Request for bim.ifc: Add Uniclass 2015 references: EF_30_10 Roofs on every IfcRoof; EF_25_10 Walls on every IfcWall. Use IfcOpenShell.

First a look at what the model holds.

```python
import ifcopenshell

model = ifcopenshell.open("bim.ifc")
print(model.schema)
print("classifications:", [c.Name for c in model.by_type("IfcClassification")])
for ifc_class in ("IfcDoor", "IfcRoof", "IfcStair", "IfcWall", "IfcWindow"):
    print(ifc_class, len(model.by_type(ifc_class)))
```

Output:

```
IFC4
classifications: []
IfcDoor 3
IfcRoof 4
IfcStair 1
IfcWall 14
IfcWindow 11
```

```python
import ifcopenshell
import ifcopenshell.api.classification

model = ifcopenshell.open("bim.ifc")

system = ifcopenshell.api.classification.add_classification(model, classification="Uniclass 2015")

codes = {
    "IfcRoof": ("EF_30_10", "Roofs"),
    "IfcWall": ("EF_25_10", "Walls"),
}
for ifc_class, (code, name) in codes.items():
    products = model.by_type(ifc_class)
    ifcopenshell.api.classification.add_reference(
        model, products=products, classification=system, identification=code, name=name
    )
    print(code, len(products))

model.write("bim_updated.ifc")
```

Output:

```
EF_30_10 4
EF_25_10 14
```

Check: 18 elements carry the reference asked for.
